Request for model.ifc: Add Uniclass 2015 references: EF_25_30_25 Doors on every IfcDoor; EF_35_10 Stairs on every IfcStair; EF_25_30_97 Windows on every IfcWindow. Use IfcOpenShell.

First a look at what the model holds.

```python
import ifcopenshell

model = ifcopenshell.open("model.ifc")
print(model.schema)
print("classifications:", [c.Name for c in model.by_type("IfcClassification")])
for ifc_class in ("IfcDoor", "IfcRoof", "IfcStair", "IfcWall", "IfcWindow"):
    print(ifc_class, len(model.by_type(ifc_class)))
```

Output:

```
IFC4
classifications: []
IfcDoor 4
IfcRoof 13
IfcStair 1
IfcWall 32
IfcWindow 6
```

```python
import ifcopenshell
import ifcopenshell.api.classification

model = ifcopenshell.open("model.ifc")

system = ifcopenshell.api.classification.add_classification(model, classification="Uniclass 2015")

codes = {
    "IfcDoor": ("EF_25_30_25", "Doors"),
    "IfcStair": ("EF_35_10", "Stairs"),
    "IfcWindow": ("EF_25_30_97", "Windows"),
}
for ifc_class, (code, name) in codes.items():
    products = model.by_type(ifc_class)
    ifcopenshell.api.classification.add_reference(
        model, products=products, classification=system, identification=code, name=name
    )
    print(code, len(products))

model.write("model_v2.ifc")
```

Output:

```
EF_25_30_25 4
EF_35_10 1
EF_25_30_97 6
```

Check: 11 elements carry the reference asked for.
